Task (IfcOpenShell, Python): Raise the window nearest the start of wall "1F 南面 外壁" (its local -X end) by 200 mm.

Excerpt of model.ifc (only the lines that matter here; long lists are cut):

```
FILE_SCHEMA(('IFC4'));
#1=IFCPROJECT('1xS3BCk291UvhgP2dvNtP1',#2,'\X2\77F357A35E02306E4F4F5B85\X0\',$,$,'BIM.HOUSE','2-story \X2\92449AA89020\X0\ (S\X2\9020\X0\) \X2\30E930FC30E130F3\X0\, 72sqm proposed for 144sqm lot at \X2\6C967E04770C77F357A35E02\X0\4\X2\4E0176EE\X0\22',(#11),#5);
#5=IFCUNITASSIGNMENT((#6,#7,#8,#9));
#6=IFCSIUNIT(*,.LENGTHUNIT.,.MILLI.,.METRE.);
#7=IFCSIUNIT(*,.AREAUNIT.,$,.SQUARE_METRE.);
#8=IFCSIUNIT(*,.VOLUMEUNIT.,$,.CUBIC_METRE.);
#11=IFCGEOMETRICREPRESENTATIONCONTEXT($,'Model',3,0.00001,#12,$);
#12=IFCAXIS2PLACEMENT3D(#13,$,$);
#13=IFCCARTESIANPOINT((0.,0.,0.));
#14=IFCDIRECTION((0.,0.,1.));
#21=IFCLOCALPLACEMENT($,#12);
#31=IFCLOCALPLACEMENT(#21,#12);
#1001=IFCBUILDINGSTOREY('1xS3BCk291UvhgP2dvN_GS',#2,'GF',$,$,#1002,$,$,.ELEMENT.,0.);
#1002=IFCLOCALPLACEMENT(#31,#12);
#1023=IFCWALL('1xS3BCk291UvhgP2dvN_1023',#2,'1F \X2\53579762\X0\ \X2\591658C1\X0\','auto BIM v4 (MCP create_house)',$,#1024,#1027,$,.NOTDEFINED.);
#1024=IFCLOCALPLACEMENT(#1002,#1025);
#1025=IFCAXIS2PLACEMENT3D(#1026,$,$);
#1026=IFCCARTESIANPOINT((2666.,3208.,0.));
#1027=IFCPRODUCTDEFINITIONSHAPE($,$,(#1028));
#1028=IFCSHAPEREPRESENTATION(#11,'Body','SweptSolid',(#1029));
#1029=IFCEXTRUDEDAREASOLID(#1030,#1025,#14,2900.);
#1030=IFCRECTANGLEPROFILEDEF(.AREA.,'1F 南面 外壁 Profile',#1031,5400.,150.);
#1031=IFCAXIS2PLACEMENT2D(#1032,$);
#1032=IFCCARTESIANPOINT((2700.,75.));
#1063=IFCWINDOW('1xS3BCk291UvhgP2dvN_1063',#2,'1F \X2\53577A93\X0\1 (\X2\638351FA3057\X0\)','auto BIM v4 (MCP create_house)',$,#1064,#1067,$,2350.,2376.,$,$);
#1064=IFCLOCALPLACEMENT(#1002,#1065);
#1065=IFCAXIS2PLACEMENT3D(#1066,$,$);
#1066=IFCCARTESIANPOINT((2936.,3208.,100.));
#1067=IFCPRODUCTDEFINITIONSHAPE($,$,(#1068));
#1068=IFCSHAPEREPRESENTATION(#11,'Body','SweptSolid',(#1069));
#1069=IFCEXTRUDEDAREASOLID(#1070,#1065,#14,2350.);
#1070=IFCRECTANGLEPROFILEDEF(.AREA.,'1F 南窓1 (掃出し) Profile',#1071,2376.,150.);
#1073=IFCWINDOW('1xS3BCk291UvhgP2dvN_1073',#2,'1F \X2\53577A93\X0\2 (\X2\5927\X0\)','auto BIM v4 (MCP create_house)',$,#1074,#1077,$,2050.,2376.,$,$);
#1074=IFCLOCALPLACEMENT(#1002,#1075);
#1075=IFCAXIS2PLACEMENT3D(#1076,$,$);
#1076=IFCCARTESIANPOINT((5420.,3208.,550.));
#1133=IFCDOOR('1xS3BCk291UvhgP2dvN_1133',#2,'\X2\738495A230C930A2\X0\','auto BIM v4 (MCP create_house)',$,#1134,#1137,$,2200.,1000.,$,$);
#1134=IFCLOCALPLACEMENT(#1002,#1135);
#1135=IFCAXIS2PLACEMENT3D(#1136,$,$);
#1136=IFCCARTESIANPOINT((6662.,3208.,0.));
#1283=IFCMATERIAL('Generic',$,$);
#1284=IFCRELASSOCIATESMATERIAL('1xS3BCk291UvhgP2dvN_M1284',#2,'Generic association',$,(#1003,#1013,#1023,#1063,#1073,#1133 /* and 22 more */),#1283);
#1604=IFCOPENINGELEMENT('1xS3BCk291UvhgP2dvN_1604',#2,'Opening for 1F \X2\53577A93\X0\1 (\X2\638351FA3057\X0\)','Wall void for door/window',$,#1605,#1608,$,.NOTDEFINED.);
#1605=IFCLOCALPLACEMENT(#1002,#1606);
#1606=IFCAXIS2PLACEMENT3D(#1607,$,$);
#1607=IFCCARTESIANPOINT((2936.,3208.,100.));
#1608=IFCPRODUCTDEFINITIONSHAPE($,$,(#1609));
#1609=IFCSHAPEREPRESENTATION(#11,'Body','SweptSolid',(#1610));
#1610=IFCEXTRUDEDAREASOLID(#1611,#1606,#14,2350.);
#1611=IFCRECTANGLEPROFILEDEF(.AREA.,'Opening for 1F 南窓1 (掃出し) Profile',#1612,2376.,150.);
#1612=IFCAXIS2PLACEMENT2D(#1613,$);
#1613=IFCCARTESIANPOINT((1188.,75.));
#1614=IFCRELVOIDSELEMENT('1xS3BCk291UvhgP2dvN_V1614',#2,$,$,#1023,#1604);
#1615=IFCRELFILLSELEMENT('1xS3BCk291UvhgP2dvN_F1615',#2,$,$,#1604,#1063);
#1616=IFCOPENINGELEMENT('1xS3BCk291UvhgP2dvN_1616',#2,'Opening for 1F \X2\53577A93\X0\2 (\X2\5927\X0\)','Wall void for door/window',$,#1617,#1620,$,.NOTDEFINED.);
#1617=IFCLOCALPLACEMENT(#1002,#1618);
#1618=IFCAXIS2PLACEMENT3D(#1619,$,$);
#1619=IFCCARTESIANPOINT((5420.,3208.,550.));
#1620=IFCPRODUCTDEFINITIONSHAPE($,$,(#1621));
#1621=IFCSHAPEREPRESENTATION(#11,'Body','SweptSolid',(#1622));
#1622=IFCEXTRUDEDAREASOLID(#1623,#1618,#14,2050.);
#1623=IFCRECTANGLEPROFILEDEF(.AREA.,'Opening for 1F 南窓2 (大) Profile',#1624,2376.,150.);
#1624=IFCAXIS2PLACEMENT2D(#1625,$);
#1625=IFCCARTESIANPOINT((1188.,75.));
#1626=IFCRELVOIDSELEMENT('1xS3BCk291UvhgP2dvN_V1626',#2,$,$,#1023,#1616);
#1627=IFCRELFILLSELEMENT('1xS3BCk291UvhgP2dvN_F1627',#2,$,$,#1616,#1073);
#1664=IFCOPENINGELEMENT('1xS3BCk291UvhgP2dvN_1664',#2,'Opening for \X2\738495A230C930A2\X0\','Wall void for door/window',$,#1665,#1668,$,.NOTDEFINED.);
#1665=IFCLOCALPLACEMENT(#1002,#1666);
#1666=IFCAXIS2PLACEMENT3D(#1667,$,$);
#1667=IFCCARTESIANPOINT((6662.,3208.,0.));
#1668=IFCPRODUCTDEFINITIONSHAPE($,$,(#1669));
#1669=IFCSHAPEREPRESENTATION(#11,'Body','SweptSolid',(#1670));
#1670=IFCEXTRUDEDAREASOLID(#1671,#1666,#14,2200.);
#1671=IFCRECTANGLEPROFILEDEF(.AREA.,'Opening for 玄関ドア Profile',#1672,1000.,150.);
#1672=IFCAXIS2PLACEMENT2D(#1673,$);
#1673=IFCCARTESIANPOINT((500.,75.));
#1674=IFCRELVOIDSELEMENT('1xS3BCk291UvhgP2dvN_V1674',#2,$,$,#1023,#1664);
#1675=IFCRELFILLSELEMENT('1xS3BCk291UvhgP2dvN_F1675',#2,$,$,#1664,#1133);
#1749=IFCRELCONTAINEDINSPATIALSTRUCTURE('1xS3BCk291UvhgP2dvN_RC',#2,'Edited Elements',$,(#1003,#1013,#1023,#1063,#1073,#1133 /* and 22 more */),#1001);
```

```python
import numpy as np
import ifcopenshell
import ifcopenshell.api.geometry
import ifcopenshell.util.placement
import ifcopenshell.util.unit

model = ifcopenshell.open("model.ifc")
unit_scale = ifcopenshell.util.unit.calculate_unit_scale(model)

window = model.by_guid("1xS3BCk291UvhgP2dvN_1063")
opening = window.FillsVoids[0].RelatingOpeningElement
dz = 200.0

shift = np.array([0.0, 0.0, dz])
# The window is not placed relative to its opening, so move both.
for product in (opening, window):
    matrix = ifcopenshell.util.placement.get_local_placement(product.ObjectPlacement)
    matrix[:3, 3] += shift
    ifcopenshell.api.geometry.edit_object_placement(model, product=product, matrix=matrix, is_si=False)

print(f"moved by {dz * unit_scale:+.3f} m")

model.write("model_edited.ifc")
```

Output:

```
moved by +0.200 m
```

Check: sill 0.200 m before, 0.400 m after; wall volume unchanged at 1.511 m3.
